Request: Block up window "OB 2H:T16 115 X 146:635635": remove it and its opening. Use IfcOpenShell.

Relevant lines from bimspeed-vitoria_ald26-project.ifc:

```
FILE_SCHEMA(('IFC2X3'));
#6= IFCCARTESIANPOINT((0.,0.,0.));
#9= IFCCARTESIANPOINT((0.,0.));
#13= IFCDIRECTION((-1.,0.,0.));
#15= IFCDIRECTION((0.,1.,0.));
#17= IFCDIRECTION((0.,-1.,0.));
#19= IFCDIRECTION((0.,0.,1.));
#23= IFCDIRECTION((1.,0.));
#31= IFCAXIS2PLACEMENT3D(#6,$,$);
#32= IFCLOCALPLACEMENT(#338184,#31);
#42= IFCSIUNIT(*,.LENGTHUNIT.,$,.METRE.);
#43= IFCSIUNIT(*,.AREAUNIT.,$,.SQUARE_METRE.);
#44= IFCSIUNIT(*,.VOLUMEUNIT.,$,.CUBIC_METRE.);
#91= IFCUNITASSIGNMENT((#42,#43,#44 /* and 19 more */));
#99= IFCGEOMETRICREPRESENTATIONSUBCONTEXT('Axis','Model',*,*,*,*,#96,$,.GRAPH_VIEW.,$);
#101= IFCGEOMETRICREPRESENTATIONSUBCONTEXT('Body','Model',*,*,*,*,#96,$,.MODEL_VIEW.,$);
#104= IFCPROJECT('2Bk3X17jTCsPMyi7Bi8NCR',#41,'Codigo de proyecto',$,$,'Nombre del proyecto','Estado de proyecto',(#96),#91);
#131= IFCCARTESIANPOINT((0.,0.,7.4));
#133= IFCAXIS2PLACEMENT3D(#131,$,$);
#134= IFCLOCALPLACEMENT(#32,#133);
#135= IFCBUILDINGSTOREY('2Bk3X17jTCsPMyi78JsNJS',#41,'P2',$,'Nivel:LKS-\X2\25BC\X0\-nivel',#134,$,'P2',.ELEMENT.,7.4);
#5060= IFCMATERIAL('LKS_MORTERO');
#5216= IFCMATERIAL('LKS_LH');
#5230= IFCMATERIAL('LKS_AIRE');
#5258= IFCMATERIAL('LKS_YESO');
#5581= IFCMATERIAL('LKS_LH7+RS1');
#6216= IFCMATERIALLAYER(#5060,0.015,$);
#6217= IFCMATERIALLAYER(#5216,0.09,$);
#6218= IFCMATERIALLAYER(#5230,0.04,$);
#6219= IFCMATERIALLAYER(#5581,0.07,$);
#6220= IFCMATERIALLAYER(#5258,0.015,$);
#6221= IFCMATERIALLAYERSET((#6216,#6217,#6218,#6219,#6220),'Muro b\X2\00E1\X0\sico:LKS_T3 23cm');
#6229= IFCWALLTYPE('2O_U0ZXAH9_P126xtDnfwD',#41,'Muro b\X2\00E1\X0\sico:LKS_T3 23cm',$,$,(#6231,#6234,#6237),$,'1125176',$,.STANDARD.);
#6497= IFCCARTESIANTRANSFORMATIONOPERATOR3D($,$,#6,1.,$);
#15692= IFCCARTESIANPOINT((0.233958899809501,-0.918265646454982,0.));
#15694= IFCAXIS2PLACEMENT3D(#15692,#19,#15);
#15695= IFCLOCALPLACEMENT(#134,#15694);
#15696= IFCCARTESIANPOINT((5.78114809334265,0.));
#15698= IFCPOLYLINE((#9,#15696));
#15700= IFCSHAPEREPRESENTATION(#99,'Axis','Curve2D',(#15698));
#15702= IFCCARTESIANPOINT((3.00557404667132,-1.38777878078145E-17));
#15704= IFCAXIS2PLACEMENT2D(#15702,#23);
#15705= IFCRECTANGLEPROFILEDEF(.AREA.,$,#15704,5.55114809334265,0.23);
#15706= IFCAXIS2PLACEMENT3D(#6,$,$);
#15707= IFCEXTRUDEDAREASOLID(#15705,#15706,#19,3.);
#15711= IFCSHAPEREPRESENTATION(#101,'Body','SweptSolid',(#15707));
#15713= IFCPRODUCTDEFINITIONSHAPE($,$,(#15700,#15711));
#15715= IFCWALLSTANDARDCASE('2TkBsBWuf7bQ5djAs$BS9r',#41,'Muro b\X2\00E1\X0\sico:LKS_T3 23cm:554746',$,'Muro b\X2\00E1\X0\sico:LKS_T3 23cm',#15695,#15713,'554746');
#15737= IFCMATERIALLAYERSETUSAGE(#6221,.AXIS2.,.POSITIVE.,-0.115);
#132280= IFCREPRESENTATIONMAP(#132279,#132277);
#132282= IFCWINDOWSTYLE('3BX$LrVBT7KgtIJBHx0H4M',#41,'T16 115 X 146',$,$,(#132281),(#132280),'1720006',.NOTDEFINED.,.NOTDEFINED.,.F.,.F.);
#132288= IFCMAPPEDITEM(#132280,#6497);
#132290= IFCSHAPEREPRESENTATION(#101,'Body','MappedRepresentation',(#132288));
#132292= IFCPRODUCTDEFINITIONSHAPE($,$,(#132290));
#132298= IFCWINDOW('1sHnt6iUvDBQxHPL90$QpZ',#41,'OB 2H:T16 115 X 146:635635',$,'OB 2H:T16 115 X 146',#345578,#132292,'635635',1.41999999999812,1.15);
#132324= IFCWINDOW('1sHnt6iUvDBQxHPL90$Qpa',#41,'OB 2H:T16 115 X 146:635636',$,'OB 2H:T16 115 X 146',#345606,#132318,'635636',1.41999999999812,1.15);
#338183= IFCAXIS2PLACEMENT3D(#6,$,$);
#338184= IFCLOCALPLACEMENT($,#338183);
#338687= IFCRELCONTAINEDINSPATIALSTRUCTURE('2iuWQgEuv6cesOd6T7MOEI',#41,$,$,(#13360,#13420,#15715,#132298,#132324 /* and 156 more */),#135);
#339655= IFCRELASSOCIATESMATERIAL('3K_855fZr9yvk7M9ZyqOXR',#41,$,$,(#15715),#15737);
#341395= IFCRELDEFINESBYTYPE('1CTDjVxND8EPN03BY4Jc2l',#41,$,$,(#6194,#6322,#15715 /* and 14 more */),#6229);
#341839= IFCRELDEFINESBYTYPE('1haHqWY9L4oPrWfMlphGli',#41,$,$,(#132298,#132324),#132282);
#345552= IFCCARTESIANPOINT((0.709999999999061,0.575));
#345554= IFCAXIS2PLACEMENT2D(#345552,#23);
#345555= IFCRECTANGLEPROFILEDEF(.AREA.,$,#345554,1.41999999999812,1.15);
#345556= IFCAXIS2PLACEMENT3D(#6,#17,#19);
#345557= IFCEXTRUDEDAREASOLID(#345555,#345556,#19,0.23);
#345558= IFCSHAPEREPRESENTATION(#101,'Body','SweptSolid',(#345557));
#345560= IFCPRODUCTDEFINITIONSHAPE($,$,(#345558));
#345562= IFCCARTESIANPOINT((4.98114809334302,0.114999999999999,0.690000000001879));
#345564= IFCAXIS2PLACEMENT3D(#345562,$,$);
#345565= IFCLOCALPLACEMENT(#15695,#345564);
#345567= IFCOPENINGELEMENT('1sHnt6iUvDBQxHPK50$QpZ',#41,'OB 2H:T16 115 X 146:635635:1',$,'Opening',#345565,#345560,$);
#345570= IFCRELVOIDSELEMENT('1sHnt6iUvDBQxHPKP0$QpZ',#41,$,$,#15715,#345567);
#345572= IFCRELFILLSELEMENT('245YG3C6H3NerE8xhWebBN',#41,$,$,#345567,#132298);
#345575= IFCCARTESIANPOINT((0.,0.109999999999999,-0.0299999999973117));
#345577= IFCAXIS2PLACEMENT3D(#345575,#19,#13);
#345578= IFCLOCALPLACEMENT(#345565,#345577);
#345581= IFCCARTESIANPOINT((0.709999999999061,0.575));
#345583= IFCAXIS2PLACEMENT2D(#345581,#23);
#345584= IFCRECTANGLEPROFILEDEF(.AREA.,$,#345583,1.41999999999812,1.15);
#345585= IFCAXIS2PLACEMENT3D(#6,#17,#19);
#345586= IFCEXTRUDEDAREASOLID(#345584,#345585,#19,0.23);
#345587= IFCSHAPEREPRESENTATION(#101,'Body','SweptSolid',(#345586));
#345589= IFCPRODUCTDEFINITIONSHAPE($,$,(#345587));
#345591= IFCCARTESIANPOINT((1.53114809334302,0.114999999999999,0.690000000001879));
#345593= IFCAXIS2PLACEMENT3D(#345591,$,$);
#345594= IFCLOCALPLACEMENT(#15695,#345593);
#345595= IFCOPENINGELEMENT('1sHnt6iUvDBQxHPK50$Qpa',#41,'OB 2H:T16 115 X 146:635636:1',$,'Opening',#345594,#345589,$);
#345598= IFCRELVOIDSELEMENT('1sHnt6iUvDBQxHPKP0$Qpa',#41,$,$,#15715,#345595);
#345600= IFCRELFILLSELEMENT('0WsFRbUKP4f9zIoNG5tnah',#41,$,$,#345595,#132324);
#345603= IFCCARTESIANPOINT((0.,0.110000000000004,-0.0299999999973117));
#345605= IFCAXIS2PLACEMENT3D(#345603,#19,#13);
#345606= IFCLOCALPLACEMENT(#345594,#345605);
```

```python
import ifcopenshell
import ifcopenshell.api.feature
import ifcopenshell.api.root
import ifcopenshell.geom
import ifcopenshell.util.shape

model = ifcopenshell.open("bimspeed-vitoria_ald26-project.ifc")
settings = ifcopenshell.geom.settings()


def volume(element):
    """Net volume in cubic metres, openings subtracted."""
    shape = ifcopenshell.geom.create_shape(settings, element)
    return ifcopenshell.util.shape.get_volume(shape.geometry)


window = model.by_guid("1sHnt6iUvDBQxHPL90$QpZ")
opening = window.FillsVoids[0].RelatingOpeningElement
wall = opening.VoidsElements[0].RelatingBuildingElement
before = volume(wall)

ifcopenshell.api.root.remove_product(model, product=window)
ifcopenshell.api.feature.remove_feature(model, feature=opening)

after = volume(wall)

print(f"wall volume {before:.3f} -> {after:.3f} m3")

model.write("bimspeed-vitoria_ald26-project_rev.ifc")
```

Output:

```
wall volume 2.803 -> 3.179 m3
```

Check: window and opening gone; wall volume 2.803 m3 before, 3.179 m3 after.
